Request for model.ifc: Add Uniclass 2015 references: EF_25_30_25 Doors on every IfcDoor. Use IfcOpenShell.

First a look at what the model holds.

```python
import ifcopenshell

model = ifcopenshell.open("model.ifc")
print(model.schema)
print("classifications:", [c.Name for c in model.by_type("IfcClassification")])
for ifc_class in ("IfcDoor", "IfcRoof", "IfcStair", "IfcWall", "IfcWindow"):
    print(ifc_class, len(model.by_type(ifc_class)))
```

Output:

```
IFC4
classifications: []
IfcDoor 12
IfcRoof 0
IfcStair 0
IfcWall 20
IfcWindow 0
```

```python
import ifcopenshell
import ifcopenshell.api.classification

model = ifcopenshell.open("model.ifc")

system = ifcopenshell.api.classification.add_classification(model, classification="Uniclass 2015")

codes = {
    "IfcDoor": ("EF_25_30_25", "Doors"),
}
for ifc_class, (code, name) in codes.items():
    products = model.by_type(ifc_class)
    ifcopenshell.api.classification.add_reference(
        model, products=products, classification=system, identification=code, name=name
    )
    print(code, len(products))

model.write("model_v2.ifc")
```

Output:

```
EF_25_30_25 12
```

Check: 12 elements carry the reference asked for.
